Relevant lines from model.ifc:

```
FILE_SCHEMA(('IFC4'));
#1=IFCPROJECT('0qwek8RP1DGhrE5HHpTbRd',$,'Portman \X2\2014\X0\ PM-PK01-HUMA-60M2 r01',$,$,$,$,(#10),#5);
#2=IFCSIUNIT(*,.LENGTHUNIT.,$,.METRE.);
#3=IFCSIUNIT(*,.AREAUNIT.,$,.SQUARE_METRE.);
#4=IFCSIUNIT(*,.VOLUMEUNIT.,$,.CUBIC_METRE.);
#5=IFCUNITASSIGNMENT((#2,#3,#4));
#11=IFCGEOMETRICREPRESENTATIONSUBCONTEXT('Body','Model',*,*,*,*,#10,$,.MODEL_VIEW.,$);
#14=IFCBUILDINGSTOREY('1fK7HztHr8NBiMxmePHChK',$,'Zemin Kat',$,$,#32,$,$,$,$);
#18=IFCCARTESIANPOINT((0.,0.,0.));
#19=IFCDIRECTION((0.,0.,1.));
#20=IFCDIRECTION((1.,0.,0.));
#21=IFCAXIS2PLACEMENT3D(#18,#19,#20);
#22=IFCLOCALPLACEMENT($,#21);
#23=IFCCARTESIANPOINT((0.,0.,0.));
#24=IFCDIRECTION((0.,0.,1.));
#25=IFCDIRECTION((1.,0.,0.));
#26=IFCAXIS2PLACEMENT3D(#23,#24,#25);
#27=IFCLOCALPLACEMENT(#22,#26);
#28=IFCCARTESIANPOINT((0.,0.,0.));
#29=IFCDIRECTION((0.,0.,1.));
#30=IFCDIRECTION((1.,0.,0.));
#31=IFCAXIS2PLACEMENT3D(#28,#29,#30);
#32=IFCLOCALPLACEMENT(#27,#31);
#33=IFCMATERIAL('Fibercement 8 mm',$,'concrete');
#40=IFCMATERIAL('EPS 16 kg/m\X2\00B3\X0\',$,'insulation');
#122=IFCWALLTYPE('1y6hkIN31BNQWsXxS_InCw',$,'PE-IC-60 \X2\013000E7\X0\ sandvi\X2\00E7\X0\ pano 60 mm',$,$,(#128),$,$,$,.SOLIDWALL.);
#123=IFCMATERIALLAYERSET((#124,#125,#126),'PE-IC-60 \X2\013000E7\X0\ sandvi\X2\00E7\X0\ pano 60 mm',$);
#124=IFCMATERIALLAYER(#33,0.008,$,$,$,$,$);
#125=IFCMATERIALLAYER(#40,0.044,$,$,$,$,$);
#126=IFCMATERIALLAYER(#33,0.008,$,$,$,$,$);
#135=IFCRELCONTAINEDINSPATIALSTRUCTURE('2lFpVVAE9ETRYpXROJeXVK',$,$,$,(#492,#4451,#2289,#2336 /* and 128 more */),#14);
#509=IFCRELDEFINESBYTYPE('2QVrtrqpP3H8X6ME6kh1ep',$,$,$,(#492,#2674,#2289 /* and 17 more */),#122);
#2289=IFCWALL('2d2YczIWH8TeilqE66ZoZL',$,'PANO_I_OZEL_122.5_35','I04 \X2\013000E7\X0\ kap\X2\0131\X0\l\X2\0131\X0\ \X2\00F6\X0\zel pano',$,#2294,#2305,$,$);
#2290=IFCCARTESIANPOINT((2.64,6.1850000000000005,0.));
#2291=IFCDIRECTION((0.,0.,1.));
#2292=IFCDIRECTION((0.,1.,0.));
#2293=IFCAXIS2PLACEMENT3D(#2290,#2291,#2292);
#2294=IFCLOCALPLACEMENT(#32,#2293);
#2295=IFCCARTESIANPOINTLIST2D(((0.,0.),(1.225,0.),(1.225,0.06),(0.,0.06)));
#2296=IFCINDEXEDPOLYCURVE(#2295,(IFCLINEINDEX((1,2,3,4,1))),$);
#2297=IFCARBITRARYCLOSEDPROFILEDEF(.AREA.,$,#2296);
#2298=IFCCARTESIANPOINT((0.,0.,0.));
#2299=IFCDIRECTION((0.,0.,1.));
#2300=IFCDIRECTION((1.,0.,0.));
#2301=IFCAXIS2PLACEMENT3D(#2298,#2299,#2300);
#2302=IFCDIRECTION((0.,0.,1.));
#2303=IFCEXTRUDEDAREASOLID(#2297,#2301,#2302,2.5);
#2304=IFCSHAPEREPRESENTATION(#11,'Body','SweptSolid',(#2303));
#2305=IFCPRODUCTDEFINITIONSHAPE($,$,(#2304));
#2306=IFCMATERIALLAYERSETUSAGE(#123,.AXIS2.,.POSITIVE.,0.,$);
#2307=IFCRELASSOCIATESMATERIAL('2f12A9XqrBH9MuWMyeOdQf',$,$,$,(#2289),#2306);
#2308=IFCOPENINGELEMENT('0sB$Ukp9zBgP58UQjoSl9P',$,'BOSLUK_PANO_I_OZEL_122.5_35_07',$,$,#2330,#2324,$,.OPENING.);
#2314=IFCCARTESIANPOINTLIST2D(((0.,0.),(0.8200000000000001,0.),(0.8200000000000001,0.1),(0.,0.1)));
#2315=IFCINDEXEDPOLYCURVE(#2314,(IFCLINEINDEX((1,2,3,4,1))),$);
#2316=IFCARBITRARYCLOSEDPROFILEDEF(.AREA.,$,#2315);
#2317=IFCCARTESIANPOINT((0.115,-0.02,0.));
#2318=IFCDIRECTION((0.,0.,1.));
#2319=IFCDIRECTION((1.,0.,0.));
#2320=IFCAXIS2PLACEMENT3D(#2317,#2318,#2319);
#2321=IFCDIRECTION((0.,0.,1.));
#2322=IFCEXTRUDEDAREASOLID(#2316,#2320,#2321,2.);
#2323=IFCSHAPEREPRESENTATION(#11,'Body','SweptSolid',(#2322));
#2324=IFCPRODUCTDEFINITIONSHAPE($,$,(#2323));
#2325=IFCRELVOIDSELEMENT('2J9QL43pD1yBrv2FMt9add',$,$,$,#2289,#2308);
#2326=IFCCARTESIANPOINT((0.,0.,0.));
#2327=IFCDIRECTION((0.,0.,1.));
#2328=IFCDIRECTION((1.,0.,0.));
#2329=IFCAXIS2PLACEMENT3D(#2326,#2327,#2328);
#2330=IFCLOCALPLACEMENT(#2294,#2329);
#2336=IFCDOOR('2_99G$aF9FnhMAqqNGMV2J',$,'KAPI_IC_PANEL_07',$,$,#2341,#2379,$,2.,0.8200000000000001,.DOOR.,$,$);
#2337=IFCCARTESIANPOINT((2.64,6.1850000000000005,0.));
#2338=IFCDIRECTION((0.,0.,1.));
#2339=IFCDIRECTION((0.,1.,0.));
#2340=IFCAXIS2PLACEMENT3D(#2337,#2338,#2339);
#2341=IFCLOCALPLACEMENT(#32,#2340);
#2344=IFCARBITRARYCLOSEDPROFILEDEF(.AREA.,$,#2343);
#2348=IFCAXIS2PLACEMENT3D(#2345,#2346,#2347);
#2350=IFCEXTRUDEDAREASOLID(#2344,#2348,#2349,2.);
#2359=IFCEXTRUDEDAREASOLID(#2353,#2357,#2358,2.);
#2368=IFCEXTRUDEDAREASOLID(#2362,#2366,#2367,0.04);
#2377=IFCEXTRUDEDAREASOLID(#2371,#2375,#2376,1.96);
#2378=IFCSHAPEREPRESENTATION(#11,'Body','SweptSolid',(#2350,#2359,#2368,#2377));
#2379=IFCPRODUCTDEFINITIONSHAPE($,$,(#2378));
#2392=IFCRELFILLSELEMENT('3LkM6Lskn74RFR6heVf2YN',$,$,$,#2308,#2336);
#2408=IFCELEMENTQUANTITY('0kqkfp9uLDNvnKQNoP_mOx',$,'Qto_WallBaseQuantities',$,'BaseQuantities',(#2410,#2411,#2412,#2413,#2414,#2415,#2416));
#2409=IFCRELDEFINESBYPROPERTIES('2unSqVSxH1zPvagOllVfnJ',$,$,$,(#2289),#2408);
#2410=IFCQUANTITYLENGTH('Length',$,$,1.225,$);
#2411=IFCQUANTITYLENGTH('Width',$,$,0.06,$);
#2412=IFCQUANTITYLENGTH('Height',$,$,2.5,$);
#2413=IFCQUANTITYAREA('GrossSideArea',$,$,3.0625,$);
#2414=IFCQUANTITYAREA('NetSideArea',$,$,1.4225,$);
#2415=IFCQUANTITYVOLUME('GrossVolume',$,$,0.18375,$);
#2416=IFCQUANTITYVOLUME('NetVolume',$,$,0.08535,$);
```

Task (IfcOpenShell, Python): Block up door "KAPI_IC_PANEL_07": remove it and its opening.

```python
import ifcopenshell
import ifcopenshell.api.feature
import ifcopenshell.api.pset
import ifcopenshell.api.root
import ifcopenshell.geom
import ifcopenshell.util.element
import ifcopenshell.util.shape
import ifcopenshell.util.unit

model = ifcopenshell.open("model.ifc")
area_scale = ifcopenshell.util.unit.calculate_unit_scale(model, "AREAUNIT")
volume_scale = ifcopenshell.util.unit.calculate_unit_scale(model, "VOLUMEUNIT")
settings = ifcopenshell.geom.settings()


def volume(element):
    """Net volume in cubic metres, openings subtracted."""
    shape = ifcopenshell.geom.create_shape(settings, element)
    return ifcopenshell.util.shape.get_volume(shape.geometry)


door = model.by_id(2336)
opening = door.FillsVoids[0].RelatingOpeningElement
wall = opening.VoidsElements[0].RelatingBuildingElement
before = volume(wall)

ifcopenshell.api.root.remove_product(model, product=door)
ifcopenshell.api.feature.remove_feature(model, feature=opening)

after = volume(wall)
thickness = 0.06  # wall thickness in metres

# Update the wall's stored quantities.
qto = model.by_id(ifcopenshell.util.element.get_pset(wall, "Qto_WallBaseQuantities", should_inherit=False)["id"])
ifcopenshell.api.pset.edit_qto(model, qto=qto, properties={
    "NetSideArea": after / thickness / area_scale,
    "NetVolume": after / volume_scale,
})

print(f"wall volume {before:.3f} -> {after:.3f} m3")

model.write("model_rev.ifc")
```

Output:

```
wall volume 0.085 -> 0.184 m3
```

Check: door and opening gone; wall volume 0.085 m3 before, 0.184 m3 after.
